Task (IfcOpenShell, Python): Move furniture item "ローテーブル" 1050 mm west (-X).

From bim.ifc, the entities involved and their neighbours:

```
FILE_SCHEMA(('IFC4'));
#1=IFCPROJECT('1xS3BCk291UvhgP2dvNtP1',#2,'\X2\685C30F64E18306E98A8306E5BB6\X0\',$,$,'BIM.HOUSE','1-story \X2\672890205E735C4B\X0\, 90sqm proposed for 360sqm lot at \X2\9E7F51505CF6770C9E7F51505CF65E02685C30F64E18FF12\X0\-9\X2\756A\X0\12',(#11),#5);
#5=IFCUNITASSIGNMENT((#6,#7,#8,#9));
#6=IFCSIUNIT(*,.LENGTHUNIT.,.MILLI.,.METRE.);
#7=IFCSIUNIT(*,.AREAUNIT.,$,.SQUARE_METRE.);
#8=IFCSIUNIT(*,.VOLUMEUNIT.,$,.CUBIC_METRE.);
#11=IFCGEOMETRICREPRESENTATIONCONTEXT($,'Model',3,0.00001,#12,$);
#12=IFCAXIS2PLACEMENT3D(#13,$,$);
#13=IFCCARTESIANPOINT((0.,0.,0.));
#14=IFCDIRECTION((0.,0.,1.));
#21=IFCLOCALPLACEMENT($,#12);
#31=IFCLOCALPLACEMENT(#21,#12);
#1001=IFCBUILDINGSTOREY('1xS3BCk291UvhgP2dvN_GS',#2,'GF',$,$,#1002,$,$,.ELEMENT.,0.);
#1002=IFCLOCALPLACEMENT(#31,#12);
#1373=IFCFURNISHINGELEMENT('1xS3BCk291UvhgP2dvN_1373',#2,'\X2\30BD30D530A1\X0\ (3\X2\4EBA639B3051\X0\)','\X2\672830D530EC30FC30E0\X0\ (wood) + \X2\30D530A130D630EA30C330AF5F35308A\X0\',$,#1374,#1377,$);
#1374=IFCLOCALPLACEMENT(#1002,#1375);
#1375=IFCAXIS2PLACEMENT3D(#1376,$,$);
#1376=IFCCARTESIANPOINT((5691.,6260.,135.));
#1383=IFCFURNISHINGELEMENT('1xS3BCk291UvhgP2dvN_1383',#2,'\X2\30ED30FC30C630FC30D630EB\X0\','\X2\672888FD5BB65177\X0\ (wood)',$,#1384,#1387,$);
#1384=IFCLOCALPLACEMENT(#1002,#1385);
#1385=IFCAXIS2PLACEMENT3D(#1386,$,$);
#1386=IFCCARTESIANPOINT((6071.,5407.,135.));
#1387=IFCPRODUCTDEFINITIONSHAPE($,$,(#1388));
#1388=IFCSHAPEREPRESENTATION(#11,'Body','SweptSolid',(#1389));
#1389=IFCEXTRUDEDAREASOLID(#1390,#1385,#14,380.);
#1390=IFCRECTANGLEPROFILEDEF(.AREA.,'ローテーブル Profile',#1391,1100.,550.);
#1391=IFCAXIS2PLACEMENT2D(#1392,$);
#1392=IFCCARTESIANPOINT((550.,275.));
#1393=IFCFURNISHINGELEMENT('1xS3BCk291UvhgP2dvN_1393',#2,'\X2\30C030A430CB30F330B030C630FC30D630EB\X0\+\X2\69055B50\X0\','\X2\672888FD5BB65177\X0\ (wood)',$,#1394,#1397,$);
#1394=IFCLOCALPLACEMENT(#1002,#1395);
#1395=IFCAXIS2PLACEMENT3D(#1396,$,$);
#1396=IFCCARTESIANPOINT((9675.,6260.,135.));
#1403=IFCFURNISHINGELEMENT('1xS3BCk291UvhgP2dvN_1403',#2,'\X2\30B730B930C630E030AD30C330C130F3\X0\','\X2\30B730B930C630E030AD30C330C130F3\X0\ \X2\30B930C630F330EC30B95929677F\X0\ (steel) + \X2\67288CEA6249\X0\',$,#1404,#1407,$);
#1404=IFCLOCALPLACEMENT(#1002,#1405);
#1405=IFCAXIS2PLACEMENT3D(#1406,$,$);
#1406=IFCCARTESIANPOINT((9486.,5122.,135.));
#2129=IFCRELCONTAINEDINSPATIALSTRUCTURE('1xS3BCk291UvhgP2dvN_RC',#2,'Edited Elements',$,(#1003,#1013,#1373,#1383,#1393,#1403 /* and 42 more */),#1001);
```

```python
import ifcopenshell
import ifcopenshell.api.geometry
import ifcopenshell.util.placement
import ifcopenshell.util.unit

model = ifcopenshell.open("bim.ifc")
unit_scale = ifcopenshell.util.unit.calculate_unit_scale(model)

item = model.by_guid("1xS3BCk291UvhgP2dvN_1383")
matrix = ifcopenshell.util.placement.get_local_placement(item.ObjectPlacement)
matrix[0, 3] -= 1.05 / unit_scale
ifcopenshell.api.geometry.edit_object_placement(model, product=item, matrix=matrix, is_si=False)

print(ifcopenshell.util.placement.get_local_placement(item.ObjectPlacement).round(3) + 0.0)

model.write("bim_rev.ifc")
```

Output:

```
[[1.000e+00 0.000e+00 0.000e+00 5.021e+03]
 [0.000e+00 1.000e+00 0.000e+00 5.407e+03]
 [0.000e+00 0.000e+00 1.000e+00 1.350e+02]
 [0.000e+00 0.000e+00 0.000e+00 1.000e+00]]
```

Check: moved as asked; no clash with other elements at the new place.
